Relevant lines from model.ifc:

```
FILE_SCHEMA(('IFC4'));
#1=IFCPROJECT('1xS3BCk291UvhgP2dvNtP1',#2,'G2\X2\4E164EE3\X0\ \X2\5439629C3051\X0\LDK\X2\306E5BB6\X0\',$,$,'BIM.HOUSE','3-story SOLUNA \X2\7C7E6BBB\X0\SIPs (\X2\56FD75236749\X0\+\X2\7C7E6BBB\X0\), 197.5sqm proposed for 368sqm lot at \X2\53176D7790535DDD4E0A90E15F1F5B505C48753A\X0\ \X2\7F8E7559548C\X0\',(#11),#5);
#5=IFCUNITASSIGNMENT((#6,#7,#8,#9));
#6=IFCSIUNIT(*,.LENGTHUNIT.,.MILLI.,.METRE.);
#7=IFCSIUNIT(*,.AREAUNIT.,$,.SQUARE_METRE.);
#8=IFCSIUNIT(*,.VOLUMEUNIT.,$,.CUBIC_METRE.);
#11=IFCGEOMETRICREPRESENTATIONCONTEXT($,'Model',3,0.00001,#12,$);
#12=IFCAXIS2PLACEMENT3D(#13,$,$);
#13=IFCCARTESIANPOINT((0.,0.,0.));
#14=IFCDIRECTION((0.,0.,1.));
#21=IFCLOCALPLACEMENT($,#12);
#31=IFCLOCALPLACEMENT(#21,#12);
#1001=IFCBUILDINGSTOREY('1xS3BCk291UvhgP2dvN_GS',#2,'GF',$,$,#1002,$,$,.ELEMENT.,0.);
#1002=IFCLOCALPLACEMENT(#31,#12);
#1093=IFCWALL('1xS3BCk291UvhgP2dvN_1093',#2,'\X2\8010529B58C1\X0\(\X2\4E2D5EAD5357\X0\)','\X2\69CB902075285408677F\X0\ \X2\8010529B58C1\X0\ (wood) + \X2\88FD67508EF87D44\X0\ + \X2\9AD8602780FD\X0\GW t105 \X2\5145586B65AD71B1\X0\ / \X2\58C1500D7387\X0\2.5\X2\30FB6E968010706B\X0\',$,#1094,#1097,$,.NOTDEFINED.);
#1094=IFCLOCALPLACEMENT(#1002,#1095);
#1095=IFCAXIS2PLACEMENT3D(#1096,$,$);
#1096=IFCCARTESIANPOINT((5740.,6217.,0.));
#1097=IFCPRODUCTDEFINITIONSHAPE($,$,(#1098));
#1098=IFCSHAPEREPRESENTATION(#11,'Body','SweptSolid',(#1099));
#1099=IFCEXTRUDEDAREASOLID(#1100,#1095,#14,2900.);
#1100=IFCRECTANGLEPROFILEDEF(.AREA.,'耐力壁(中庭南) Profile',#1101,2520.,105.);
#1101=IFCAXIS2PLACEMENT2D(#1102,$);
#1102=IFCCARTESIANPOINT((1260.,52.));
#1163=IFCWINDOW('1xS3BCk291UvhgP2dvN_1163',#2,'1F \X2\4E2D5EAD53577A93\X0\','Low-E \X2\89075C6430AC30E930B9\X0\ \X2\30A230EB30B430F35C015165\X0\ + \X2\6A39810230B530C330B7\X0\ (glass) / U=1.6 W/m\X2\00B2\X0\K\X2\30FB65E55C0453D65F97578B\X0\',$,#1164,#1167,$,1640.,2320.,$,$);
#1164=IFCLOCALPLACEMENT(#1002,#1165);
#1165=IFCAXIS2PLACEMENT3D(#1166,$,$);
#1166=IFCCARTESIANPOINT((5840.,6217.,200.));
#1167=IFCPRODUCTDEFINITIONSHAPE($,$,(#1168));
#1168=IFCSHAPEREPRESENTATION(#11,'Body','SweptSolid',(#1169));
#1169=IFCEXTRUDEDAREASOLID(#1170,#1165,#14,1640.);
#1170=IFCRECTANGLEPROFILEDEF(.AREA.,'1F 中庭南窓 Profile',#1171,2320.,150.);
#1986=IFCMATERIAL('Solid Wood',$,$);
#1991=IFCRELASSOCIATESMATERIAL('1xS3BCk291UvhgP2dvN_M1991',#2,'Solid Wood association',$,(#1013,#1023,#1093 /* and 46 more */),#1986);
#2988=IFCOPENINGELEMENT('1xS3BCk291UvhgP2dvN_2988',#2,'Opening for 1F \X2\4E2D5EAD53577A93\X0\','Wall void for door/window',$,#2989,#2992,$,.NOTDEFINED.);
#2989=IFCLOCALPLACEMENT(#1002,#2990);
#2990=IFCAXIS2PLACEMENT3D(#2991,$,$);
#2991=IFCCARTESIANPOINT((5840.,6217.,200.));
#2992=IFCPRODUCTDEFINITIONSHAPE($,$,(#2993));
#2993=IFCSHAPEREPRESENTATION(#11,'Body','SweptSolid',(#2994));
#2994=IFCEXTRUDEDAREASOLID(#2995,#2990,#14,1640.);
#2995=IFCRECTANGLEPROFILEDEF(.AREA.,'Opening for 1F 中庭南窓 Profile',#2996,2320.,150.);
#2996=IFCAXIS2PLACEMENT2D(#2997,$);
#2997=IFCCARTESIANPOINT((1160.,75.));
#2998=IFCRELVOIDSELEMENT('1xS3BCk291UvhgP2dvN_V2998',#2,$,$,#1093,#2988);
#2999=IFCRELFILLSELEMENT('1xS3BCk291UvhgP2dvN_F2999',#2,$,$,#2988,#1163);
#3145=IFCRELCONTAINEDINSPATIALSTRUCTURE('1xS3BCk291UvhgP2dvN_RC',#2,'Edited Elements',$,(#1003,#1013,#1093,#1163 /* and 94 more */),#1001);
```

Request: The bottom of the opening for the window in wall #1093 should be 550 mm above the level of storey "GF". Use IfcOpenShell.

```python
import numpy as np
import ifcopenshell
import ifcopenshell.api.geometry
import ifcopenshell.geom
import ifcopenshell.util.element
import ifcopenshell.util.placement
import ifcopenshell.util.shape
import ifcopenshell.util.unit

model = ifcopenshell.open("model.ifc")
unit_scale = ifcopenshell.util.unit.calculate_unit_scale(model)

window = model.by_guid("1xS3BCk291UvhgP2dvN_1163")
opening = window.FillsVoids[0].RelatingOpeningElement
storey = ifcopenshell.util.element.get_container(window, ifc_class="IfcBuildingStorey")
level = ifcopenshell.util.placement.get_local_placement(storey.ObjectPlacement)[2, 3]

# The opening's origin need not be at the sill, so measure its lowest point.
shape = ifcopenshell.geom.create_shape(ifcopenshell.geom.settings(), opening)
bottom = ifcopenshell.util.shape.get_shape_bottom_elevation(shape, shape.geometry) / unit_scale
dz = level + 0.55 / unit_scale - bottom

shift = np.array([0.0, 0.0, dz])
# The window is not placed relative to its opening, so move both.
for product in (opening, window):
    matrix = ifcopenshell.util.placement.get_local_placement(product.ObjectPlacement)
    matrix[:3, 3] += shift
    ifcopenshell.api.geometry.edit_object_placement(model, product=product, matrix=matrix, is_si=False)

print(f"moved by {dz * unit_scale:+.3f} m")

model.write("model_rev.ifc")
```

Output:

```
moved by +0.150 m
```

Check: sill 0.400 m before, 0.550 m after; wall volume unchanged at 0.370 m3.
